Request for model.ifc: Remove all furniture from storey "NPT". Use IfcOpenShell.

First a look at what the model holds.

```python
import ifcopenshell
import ifcopenshell.util.element

model = ifcopenshell.open("model.ifc")
print(model.schema)
storey = next(s for s in model.by_type("IfcBuildingStorey") if s.Name == "NPT")
furniture = [e for e in ifcopenshell.util.element.get_decomposition(storey) if e.is_a("IfcFurnishingElement")]
seen = {}
for e in furniture:
    element_type = ifcopenshell.util.element.get_type(e)
    name = element_type.Name if element_type not in (None, e) else None
    seen[name] = seen.get(name, 0) + 1
for name, count in sorted(seen.items(), key=str):
    print(count, "x", name)
```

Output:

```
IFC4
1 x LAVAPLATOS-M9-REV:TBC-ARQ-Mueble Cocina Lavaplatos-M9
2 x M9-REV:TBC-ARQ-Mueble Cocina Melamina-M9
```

```python
import ifcopenshell
import ifcopenshell.api.root
import ifcopenshell.util.element

model = ifcopenshell.open("model.ifc")

storey = next(s for s in model.by_type("IfcBuildingStorey") if s.Name == "NPT")
furniture = [e for e in ifcopenshell.util.element.get_decomposition(storey) if e.is_a("IfcFurnishingElement")]

for e in furniture:
    ifcopenshell.api.root.remove_product(model, product=e)
print(len(furniture), "removed")

model.write("model-out.ifc")
```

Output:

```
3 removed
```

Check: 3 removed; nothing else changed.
